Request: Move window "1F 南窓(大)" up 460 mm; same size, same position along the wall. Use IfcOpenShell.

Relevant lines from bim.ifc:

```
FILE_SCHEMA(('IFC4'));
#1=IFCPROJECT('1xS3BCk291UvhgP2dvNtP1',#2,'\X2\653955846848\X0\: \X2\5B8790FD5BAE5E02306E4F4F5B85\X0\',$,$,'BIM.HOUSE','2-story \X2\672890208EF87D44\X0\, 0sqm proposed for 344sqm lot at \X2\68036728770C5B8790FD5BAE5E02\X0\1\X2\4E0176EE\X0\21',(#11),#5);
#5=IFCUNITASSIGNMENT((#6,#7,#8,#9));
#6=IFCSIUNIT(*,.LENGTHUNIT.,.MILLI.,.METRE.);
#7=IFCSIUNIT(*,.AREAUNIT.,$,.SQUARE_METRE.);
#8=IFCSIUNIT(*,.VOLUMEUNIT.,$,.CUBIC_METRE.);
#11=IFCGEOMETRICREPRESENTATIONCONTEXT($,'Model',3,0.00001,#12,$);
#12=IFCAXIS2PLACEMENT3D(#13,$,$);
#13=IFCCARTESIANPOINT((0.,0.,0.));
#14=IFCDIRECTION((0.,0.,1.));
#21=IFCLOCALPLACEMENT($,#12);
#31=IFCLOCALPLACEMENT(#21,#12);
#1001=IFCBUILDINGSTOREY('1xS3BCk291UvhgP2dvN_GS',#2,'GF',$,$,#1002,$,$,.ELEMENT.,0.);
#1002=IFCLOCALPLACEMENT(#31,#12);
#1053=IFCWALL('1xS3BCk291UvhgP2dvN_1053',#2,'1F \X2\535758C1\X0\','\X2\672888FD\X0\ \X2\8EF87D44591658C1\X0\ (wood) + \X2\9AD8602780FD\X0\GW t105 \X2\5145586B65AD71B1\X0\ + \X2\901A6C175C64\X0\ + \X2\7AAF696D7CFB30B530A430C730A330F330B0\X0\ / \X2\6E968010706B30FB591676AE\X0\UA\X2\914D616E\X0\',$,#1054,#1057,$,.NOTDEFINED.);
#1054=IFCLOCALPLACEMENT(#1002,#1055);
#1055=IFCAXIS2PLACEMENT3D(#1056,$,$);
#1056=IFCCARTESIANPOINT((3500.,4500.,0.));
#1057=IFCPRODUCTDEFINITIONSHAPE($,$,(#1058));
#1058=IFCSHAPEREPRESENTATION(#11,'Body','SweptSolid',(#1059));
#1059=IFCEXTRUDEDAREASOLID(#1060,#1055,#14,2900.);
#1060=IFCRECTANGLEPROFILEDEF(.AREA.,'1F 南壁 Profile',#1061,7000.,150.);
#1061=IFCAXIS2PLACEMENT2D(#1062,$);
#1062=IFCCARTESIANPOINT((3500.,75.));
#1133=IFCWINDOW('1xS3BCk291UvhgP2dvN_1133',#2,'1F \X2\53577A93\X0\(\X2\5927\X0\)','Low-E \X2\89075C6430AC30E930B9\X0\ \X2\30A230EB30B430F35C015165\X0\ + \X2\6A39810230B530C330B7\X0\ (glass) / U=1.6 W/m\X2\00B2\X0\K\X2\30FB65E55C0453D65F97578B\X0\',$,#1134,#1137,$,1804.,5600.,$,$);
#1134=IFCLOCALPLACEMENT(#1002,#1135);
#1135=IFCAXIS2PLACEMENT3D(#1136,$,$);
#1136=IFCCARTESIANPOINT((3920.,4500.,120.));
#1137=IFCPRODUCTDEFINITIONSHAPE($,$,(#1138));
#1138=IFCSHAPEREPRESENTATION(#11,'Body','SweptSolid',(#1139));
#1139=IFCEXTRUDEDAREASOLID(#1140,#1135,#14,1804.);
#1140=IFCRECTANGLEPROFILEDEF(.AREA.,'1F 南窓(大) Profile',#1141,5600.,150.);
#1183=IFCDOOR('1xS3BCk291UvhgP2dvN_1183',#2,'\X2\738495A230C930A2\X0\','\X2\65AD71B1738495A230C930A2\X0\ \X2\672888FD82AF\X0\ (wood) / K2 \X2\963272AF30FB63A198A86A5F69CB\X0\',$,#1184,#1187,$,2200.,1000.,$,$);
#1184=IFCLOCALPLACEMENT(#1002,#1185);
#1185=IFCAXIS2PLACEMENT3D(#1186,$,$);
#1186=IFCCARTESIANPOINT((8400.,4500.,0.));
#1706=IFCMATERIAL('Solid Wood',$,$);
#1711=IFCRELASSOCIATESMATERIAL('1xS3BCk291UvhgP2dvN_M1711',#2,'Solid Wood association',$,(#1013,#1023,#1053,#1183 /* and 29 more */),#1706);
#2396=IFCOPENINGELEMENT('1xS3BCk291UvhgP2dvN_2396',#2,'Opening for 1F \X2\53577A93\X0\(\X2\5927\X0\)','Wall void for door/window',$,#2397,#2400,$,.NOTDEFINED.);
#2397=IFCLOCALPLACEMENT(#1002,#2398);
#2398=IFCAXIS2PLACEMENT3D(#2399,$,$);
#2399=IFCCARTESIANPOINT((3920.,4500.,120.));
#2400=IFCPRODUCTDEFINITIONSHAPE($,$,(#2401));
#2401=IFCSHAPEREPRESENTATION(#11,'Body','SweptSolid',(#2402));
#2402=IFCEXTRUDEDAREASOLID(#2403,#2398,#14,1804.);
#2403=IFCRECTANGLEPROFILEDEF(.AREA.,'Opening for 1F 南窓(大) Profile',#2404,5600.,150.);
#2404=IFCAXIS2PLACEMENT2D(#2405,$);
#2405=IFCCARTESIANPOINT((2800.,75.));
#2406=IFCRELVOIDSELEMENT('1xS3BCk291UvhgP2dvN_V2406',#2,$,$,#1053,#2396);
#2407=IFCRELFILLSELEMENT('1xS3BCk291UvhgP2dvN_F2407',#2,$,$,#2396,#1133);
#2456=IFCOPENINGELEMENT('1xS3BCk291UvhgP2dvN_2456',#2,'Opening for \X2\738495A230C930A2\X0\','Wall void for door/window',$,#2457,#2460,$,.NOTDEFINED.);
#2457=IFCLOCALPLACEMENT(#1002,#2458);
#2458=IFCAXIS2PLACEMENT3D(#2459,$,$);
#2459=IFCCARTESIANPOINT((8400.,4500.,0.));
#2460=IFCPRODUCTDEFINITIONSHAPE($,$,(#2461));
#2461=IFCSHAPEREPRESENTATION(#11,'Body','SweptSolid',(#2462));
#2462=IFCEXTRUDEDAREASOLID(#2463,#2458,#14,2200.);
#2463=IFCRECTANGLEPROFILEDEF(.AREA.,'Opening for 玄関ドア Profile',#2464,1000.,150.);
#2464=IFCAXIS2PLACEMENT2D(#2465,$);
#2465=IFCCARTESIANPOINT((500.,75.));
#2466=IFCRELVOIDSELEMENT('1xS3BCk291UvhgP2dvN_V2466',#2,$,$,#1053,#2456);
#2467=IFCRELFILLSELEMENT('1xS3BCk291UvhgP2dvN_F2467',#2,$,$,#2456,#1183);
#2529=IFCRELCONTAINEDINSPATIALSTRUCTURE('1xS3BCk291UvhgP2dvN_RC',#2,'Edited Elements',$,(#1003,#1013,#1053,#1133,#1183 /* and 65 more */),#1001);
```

```python
import numpy as np
import ifcopenshell
import ifcopenshell.api.geometry
import ifcopenshell.util.placement
import ifcopenshell.util.unit

model = ifcopenshell.open("bim.ifc")
unit_scale = ifcopenshell.util.unit.calculate_unit_scale(model)

window = model.by_guid("1xS3BCk291UvhgP2dvN_1133")
opening = window.FillsVoids[0].RelatingOpeningElement
dz = 0.46 / unit_scale

shift = np.array([0.0, 0.0, dz])
# The window is not placed relative to its opening, so move both.
for product in (opening, window):
    matrix = ifcopenshell.util.placement.get_local_placement(product.ObjectPlacement)
    matrix[:3, 3] += shift
    ifcopenshell.api.geometry.edit_object_placement(model, product=product, matrix=matrix, is_si=False)

print(f"moved by {dz * unit_scale:+.3f} m")

model.write("bim_rev.ifc")
```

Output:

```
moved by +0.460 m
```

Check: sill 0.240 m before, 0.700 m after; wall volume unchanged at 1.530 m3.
